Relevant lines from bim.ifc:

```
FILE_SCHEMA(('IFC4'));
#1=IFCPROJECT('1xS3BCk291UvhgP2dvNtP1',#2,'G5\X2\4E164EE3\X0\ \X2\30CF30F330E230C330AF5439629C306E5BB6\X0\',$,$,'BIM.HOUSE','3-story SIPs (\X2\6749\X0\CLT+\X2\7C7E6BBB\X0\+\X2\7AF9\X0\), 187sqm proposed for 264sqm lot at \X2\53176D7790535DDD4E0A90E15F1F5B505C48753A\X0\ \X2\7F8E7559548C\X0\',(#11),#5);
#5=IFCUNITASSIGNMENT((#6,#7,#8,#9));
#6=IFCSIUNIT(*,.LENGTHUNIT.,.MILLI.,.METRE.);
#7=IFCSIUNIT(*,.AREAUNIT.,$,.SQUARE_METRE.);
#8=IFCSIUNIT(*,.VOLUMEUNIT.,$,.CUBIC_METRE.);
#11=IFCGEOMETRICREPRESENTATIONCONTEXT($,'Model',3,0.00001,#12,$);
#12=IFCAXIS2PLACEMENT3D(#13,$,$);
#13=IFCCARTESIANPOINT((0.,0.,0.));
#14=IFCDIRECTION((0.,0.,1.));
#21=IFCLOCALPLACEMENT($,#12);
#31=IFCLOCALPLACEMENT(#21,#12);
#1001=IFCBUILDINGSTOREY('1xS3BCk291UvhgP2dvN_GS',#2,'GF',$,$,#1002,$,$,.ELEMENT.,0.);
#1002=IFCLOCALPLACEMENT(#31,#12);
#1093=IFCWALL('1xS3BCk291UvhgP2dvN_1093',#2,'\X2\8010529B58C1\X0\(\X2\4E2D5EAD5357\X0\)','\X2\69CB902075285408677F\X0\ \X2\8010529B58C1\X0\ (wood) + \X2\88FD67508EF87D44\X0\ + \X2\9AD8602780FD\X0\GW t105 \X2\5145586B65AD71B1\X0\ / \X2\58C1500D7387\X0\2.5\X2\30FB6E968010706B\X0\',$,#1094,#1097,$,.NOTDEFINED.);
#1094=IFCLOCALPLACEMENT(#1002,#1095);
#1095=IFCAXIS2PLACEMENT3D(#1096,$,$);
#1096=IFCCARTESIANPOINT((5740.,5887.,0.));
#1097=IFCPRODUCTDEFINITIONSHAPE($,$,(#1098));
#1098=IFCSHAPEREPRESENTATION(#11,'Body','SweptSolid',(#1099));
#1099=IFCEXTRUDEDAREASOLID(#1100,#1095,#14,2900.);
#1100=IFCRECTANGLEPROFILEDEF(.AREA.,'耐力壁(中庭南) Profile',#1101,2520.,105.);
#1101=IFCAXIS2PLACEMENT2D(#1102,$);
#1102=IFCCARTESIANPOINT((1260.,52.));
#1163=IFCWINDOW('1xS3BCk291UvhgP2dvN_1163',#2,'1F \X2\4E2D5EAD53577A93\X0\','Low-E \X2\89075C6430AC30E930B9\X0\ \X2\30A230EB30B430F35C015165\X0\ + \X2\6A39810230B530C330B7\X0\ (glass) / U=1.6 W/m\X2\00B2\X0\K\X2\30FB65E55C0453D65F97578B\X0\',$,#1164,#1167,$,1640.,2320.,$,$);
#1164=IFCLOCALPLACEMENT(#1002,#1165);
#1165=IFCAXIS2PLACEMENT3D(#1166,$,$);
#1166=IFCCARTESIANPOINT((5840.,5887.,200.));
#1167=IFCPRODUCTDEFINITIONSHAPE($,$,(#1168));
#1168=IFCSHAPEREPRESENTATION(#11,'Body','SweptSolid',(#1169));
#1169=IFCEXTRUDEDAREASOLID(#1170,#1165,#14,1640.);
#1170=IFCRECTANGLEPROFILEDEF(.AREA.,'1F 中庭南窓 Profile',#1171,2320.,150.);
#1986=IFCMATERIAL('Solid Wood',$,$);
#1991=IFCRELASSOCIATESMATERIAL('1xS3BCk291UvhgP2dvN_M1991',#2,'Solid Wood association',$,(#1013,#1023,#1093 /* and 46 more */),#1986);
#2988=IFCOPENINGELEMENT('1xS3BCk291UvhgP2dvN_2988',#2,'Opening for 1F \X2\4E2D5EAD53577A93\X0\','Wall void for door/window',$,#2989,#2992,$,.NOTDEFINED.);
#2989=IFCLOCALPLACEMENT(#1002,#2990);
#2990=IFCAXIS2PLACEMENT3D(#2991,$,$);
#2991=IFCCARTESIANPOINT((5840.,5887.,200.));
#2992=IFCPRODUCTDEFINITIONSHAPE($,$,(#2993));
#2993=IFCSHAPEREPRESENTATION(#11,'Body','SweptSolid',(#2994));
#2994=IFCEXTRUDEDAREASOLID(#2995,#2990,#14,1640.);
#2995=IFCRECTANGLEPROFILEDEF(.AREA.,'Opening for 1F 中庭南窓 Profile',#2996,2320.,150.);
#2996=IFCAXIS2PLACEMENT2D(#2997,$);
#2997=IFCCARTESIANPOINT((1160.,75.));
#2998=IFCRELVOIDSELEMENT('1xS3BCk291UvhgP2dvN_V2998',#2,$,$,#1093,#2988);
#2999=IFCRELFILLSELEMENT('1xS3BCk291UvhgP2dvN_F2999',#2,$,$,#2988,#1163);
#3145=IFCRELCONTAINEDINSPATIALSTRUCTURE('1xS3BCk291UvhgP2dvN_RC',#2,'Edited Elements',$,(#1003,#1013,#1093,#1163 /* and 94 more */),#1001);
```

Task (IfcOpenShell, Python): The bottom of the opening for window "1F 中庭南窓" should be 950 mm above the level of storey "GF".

```python
import numpy as np
import ifcopenshell
import ifcopenshell.api.geometry
import ifcopenshell.geom
import ifcopenshell.util.element
import ifcopenshell.util.placement
import ifcopenshell.util.shape
import ifcopenshell.util.unit

model = ifcopenshell.open("bim.ifc")
unit_scale = ifcopenshell.util.unit.calculate_unit_scale(model)

window = model.by_guid("1xS3BCk291UvhgP2dvN_1163")
opening = window.FillsVoids[0].RelatingOpeningElement
storey = ifcopenshell.util.element.get_container(window, ifc_class="IfcBuildingStorey")
level = ifcopenshell.util.placement.get_local_placement(storey.ObjectPlacement)[2, 3]

# The opening's origin need not be at the sill, so measure its lowest point.
shape = ifcopenshell.geom.create_shape(ifcopenshell.geom.settings(), opening)
bottom = ifcopenshell.util.shape.get_shape_bottom_elevation(shape, shape.geometry) / unit_scale
dz = level + 950.0 - bottom

shift = np.array([0.0, 0.0, dz])
# The window is not placed relative to its opening, so move both.
for product in (opening, window):
    matrix = ifcopenshell.util.placement.get_local_placement(product.ObjectPlacement)
    matrix[:3, 3] += shift
    ifcopenshell.api.geometry.edit_object_placement(model, product=product, matrix=matrix, is_si=False)

print(f"moved by {dz * unit_scale:+.3f} m")

model.write("bim-out.ifc")
```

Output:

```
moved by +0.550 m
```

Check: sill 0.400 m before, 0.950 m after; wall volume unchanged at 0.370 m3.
